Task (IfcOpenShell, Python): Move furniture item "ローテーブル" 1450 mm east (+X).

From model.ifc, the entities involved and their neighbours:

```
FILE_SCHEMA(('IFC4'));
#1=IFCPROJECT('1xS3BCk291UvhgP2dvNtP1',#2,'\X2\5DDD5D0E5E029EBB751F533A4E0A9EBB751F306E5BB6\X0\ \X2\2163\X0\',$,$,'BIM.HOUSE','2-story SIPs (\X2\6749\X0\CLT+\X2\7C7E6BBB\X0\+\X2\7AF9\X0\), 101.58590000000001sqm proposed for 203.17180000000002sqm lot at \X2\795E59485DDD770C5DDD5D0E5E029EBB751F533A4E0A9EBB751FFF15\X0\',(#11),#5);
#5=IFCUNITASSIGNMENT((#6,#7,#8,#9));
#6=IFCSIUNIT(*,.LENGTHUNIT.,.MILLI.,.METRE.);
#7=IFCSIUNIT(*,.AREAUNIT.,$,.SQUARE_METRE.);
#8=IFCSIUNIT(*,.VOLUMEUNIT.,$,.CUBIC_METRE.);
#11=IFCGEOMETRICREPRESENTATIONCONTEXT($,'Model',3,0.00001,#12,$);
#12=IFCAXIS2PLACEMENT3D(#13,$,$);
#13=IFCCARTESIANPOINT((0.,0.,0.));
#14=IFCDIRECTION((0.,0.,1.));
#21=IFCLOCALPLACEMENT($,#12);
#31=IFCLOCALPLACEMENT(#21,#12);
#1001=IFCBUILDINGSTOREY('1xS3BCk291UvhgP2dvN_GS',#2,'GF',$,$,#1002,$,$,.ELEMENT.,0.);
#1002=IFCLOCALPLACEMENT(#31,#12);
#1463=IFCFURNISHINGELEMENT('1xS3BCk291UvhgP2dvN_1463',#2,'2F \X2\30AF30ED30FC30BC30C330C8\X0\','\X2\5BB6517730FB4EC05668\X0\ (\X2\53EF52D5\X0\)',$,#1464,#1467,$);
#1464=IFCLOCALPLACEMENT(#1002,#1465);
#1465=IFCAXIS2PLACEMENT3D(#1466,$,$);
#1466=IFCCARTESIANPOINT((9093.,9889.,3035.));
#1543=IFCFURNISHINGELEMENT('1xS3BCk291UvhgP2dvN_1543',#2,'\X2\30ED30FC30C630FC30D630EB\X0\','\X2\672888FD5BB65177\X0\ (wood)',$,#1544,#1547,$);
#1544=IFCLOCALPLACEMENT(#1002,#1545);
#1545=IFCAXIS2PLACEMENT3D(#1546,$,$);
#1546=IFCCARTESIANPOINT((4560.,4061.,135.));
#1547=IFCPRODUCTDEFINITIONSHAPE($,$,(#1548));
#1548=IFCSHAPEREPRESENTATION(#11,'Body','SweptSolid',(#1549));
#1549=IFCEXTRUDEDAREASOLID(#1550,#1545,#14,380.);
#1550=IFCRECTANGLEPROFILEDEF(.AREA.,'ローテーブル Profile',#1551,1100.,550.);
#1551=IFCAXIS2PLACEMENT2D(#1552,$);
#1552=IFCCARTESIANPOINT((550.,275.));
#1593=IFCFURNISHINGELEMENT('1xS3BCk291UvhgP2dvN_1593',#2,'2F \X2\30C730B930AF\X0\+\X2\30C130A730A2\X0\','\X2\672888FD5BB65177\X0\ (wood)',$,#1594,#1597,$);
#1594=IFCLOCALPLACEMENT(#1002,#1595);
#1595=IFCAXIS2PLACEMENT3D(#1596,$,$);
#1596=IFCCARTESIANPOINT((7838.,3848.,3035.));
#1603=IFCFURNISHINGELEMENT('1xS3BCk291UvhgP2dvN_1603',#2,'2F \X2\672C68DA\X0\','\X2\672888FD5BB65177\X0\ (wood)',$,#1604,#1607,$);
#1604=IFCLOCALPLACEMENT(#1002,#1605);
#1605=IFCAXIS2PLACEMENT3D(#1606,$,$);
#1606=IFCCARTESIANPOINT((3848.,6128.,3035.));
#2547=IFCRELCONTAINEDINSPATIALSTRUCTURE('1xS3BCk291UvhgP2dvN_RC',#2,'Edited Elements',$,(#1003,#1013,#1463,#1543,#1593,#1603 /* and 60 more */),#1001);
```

```python
import ifcopenshell
import ifcopenshell.api.geometry
import ifcopenshell.util.placement

model = ifcopenshell.open("model.ifc")

item = model.by_id(1543)
matrix = ifcopenshell.util.placement.get_local_placement(item.ObjectPlacement)
matrix[0, 3] += 1450.0
ifcopenshell.api.geometry.edit_object_placement(model, product=item, matrix=matrix, is_si=False)

print(ifcopenshell.util.placement.get_local_placement(item.ObjectPlacement).round(3) + 0.0)

model.write("model_rev.ifc")
```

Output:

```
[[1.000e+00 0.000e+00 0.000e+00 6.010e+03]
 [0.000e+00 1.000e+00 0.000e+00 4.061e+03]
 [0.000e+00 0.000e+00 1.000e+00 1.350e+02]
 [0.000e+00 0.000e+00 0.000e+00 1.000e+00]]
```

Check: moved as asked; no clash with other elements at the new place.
